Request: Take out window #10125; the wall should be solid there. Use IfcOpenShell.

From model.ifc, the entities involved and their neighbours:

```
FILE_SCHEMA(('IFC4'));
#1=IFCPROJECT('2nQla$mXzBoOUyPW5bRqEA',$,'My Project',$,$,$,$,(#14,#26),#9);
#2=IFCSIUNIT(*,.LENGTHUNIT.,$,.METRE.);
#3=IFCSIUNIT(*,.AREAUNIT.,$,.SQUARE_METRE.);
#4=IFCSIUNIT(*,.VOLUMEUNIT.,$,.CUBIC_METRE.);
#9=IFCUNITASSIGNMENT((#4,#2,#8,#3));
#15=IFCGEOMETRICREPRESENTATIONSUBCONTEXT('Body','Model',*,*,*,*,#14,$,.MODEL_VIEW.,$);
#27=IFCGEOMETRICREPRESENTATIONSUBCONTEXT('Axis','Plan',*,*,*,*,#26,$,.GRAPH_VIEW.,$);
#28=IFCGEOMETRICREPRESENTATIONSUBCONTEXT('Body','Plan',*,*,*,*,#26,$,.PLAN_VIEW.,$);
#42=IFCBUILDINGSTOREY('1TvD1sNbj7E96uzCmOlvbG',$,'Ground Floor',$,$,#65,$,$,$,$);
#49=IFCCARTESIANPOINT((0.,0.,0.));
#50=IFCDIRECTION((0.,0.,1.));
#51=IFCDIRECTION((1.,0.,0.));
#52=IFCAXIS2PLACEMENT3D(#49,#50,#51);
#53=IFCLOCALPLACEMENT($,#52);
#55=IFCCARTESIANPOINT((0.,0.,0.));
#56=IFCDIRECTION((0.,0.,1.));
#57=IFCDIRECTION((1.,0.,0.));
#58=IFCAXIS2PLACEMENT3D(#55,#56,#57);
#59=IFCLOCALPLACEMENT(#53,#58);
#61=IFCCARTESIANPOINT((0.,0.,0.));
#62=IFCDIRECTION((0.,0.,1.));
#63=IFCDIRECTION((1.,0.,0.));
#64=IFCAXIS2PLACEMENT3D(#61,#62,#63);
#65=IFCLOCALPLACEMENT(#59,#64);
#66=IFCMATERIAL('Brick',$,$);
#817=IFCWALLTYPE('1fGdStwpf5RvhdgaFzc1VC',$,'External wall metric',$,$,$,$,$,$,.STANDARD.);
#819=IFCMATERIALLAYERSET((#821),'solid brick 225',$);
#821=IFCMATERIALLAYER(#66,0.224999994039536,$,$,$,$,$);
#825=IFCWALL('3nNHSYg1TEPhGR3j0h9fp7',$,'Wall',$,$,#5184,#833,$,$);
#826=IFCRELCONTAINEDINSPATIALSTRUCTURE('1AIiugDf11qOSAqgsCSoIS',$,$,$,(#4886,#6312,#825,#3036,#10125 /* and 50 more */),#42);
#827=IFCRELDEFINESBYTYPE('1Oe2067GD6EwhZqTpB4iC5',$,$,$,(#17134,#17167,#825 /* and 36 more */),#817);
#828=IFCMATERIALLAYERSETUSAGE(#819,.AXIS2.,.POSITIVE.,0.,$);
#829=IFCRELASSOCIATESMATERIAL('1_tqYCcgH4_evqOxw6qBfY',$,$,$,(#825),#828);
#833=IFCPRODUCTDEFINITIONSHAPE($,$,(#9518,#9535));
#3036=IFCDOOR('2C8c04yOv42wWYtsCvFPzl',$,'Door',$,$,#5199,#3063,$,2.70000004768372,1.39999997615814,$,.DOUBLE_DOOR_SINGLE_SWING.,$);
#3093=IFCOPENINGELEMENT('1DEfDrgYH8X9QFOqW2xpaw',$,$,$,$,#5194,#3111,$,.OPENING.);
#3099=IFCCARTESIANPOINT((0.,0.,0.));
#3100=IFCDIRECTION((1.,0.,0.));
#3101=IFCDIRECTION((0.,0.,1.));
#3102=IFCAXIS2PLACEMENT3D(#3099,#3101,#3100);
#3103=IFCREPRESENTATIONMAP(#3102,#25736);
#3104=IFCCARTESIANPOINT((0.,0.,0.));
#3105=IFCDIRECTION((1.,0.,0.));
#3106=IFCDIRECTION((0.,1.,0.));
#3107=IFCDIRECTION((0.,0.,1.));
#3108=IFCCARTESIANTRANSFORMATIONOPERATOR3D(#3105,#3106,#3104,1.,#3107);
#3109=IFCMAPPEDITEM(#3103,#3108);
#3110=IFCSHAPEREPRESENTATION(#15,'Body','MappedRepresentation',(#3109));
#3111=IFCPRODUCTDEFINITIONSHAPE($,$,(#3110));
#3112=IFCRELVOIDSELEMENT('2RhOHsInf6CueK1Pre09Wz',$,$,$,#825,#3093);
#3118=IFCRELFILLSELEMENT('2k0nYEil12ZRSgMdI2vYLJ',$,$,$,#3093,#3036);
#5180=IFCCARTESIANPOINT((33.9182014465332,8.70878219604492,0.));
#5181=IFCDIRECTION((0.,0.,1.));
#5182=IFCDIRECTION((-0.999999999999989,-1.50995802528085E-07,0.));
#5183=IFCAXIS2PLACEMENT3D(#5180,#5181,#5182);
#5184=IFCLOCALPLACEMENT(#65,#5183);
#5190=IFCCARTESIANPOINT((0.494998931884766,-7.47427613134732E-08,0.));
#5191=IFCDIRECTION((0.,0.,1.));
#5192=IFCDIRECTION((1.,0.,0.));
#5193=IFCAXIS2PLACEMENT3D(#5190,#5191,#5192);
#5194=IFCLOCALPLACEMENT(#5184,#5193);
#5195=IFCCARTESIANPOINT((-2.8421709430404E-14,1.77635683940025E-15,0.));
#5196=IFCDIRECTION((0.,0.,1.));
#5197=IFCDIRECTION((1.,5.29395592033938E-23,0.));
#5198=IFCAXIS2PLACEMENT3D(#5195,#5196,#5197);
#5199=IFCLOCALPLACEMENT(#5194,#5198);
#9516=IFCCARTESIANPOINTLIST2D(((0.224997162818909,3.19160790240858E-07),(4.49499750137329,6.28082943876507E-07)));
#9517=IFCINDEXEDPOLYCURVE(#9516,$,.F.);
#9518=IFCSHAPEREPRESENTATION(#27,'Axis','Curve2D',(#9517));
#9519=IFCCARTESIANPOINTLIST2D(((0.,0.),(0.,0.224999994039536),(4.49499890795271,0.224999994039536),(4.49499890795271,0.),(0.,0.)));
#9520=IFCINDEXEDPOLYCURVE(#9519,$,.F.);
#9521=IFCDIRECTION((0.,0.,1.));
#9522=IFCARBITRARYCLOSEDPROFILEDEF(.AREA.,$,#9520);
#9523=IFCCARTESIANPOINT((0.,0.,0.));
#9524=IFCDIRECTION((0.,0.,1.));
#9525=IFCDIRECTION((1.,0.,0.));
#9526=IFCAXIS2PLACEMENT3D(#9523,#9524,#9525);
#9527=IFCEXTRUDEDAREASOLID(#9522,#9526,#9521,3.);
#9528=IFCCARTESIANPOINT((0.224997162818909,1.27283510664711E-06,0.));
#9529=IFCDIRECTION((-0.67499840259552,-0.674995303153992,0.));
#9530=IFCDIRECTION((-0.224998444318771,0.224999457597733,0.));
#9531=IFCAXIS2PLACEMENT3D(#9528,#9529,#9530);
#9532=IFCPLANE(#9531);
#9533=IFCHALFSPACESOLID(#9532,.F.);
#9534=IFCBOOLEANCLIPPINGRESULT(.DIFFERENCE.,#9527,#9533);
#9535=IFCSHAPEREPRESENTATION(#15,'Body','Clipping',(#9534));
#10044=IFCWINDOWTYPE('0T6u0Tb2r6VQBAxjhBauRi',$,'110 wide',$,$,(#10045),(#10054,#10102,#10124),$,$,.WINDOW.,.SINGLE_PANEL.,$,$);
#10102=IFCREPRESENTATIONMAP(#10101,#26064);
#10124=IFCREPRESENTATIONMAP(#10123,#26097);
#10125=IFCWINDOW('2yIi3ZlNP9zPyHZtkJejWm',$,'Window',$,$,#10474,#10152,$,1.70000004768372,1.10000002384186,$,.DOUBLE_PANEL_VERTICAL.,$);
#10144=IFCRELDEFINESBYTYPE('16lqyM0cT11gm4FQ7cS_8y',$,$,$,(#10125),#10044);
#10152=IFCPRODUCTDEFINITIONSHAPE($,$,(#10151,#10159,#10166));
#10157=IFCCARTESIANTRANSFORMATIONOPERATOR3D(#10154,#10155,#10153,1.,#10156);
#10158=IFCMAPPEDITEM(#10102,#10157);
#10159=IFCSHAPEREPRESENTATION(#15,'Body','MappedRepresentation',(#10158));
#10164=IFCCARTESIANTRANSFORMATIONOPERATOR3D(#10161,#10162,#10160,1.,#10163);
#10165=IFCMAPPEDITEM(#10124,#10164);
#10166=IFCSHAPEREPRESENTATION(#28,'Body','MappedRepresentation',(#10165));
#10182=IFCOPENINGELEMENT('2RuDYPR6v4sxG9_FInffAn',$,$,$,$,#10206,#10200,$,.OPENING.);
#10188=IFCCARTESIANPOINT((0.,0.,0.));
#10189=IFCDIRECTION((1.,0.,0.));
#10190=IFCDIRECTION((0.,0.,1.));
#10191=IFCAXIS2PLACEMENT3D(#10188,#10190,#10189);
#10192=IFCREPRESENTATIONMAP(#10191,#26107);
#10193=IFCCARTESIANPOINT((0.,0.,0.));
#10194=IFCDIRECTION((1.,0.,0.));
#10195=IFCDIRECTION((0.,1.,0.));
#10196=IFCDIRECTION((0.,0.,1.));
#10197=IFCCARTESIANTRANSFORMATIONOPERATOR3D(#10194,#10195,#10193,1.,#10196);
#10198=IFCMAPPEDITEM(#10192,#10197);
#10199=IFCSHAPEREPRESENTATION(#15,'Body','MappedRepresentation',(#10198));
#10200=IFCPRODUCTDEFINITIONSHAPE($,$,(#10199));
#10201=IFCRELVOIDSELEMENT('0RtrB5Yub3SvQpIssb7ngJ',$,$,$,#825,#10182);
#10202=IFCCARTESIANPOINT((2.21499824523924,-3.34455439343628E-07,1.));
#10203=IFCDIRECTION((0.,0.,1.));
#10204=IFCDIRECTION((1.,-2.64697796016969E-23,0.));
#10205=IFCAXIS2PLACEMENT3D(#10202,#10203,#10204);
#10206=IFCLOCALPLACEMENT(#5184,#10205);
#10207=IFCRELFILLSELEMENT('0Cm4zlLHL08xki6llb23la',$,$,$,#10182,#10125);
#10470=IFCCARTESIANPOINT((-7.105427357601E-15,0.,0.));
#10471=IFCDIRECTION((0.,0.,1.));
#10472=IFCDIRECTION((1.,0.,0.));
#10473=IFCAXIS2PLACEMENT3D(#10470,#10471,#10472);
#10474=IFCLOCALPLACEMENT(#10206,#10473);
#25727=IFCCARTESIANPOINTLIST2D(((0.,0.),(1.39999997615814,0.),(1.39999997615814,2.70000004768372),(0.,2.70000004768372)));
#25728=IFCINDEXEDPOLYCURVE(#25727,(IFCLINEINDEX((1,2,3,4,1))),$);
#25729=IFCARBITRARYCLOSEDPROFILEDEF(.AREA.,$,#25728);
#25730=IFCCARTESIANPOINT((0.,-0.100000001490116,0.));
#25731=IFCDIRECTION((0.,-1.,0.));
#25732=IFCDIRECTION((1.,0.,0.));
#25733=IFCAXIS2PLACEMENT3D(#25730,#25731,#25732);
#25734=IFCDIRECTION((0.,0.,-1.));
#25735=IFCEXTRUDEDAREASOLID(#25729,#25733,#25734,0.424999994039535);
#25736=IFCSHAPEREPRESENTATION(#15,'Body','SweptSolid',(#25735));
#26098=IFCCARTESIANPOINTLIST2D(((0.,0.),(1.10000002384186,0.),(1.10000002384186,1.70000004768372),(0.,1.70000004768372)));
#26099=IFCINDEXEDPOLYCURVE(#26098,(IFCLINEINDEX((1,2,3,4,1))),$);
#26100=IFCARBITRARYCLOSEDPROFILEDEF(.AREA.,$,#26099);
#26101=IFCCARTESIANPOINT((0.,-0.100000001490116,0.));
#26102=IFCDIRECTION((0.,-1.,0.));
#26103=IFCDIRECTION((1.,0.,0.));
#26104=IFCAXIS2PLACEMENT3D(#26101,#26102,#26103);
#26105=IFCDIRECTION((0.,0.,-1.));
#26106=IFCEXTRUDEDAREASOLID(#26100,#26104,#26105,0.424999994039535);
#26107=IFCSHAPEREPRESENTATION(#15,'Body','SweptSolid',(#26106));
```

```python
import ifcopenshell
import ifcopenshell.api.feature
import ifcopenshell.api.root
import ifcopenshell.geom
import ifcopenshell.util.shape

model = ifcopenshell.open("model.ifc")
settings = ifcopenshell.geom.settings()


def volume(element):
    """Net volume in cubic metres, openings subtracted."""
    shape = ifcopenshell.geom.create_shape(settings, element)
    return ifcopenshell.util.shape.get_volume(shape.geometry)


window = model.by_guid("2yIi3ZlNP9zPyHZtkJejWm")
opening = window.FillsVoids[0].RelatingOpeningElement
wall = opening.VoidsElements[0].RelatingBuildingElement
before = volume(wall)

ifcopenshell.api.root.remove_product(model, product=window)
ifcopenshell.api.feature.remove_feature(model, feature=opening)

after = volume(wall)

print(f"wall volume {before:.3f} -> {after:.3f} m3")

model.write("model-out.ifc")
```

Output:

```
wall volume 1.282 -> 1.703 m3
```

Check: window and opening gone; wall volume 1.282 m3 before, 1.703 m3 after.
